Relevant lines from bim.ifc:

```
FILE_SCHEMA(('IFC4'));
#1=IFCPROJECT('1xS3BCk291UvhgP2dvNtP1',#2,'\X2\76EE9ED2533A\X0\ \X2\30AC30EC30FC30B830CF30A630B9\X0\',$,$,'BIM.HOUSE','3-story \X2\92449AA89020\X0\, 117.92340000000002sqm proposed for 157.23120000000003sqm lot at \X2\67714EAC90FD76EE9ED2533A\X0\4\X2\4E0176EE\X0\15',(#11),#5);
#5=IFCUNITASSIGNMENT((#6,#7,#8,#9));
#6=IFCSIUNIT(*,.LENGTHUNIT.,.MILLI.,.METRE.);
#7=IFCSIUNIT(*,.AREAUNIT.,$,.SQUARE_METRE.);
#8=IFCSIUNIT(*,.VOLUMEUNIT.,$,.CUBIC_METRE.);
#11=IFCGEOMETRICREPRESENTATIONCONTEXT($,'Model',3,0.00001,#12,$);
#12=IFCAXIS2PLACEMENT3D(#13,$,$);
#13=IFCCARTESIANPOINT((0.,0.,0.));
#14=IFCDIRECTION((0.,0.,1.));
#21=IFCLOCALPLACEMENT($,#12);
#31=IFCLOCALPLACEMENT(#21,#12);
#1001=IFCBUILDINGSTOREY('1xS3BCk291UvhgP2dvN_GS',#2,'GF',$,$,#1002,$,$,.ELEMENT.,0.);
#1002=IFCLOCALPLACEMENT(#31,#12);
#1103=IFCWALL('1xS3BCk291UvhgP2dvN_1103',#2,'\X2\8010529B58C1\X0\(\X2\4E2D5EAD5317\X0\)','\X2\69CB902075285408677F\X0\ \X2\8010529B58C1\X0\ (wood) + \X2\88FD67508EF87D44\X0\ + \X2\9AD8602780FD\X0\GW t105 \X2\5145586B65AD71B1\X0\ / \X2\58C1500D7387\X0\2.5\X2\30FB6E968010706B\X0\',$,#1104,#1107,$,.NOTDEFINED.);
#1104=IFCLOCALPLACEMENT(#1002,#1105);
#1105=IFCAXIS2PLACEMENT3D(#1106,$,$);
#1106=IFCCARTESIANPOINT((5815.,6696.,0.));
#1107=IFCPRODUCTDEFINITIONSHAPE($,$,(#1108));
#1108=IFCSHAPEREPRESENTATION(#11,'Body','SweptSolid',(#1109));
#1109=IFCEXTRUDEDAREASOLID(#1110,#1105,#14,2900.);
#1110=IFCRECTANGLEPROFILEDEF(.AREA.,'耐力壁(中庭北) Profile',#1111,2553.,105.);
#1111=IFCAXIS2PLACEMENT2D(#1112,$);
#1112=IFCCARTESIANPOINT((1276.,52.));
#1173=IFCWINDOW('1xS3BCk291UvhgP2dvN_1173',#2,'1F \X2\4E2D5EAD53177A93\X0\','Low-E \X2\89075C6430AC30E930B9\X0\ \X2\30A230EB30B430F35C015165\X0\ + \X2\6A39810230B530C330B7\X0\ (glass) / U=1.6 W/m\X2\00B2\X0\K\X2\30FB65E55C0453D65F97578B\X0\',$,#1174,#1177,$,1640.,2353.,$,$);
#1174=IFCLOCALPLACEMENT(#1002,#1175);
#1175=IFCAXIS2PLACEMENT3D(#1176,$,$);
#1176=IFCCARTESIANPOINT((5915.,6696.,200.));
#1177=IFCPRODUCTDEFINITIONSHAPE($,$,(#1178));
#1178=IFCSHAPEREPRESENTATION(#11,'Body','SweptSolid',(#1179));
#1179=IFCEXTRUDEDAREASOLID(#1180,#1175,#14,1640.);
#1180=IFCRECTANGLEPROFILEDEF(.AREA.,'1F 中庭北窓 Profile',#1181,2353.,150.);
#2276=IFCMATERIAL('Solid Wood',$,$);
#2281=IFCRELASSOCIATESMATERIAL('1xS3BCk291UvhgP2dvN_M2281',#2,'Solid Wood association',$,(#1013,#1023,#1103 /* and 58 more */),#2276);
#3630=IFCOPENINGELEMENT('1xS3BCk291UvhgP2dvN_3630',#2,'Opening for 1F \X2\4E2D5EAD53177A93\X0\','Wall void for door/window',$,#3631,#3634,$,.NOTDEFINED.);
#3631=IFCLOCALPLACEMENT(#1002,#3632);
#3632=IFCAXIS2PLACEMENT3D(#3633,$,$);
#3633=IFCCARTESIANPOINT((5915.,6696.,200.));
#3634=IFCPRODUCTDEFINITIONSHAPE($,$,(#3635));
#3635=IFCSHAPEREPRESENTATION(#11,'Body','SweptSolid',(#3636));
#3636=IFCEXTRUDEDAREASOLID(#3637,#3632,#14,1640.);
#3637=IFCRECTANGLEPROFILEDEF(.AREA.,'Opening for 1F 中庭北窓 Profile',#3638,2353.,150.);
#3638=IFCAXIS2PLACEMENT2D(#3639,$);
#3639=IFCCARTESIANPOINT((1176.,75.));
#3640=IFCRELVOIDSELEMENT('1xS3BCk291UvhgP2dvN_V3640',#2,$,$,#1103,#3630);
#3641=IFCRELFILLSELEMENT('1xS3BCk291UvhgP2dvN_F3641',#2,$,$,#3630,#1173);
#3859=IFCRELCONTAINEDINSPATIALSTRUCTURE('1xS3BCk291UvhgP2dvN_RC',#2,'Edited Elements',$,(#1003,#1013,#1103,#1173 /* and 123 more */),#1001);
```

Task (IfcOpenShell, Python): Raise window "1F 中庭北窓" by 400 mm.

```python
import numpy as np
import ifcopenshell
import ifcopenshell.api.geometry
import ifcopenshell.util.placement
import ifcopenshell.util.unit

model = ifcopenshell.open("bim.ifc")
unit_scale = ifcopenshell.util.unit.calculate_unit_scale(model)

window = model.by_guid("1xS3BCk291UvhgP2dvN_1173")
opening = window.FillsVoids[0].RelatingOpeningElement
dz = 0.4 / unit_scale

shift = np.array([0.0, 0.0, dz])
# The window is not placed relative to its opening, so move both.
for product in (opening, window):
    matrix = ifcopenshell.util.placement.get_local_placement(product.ObjectPlacement)
    matrix[:3, 3] += shift
    ifcopenshell.api.geometry.edit_object_placement(model, product=product, matrix=matrix, is_si=False)

print(f"moved by {dz * unit_scale:+.3f} m")

model.write("bim_v2.ifc")
```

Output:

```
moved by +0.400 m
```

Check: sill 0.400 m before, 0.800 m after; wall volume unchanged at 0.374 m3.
